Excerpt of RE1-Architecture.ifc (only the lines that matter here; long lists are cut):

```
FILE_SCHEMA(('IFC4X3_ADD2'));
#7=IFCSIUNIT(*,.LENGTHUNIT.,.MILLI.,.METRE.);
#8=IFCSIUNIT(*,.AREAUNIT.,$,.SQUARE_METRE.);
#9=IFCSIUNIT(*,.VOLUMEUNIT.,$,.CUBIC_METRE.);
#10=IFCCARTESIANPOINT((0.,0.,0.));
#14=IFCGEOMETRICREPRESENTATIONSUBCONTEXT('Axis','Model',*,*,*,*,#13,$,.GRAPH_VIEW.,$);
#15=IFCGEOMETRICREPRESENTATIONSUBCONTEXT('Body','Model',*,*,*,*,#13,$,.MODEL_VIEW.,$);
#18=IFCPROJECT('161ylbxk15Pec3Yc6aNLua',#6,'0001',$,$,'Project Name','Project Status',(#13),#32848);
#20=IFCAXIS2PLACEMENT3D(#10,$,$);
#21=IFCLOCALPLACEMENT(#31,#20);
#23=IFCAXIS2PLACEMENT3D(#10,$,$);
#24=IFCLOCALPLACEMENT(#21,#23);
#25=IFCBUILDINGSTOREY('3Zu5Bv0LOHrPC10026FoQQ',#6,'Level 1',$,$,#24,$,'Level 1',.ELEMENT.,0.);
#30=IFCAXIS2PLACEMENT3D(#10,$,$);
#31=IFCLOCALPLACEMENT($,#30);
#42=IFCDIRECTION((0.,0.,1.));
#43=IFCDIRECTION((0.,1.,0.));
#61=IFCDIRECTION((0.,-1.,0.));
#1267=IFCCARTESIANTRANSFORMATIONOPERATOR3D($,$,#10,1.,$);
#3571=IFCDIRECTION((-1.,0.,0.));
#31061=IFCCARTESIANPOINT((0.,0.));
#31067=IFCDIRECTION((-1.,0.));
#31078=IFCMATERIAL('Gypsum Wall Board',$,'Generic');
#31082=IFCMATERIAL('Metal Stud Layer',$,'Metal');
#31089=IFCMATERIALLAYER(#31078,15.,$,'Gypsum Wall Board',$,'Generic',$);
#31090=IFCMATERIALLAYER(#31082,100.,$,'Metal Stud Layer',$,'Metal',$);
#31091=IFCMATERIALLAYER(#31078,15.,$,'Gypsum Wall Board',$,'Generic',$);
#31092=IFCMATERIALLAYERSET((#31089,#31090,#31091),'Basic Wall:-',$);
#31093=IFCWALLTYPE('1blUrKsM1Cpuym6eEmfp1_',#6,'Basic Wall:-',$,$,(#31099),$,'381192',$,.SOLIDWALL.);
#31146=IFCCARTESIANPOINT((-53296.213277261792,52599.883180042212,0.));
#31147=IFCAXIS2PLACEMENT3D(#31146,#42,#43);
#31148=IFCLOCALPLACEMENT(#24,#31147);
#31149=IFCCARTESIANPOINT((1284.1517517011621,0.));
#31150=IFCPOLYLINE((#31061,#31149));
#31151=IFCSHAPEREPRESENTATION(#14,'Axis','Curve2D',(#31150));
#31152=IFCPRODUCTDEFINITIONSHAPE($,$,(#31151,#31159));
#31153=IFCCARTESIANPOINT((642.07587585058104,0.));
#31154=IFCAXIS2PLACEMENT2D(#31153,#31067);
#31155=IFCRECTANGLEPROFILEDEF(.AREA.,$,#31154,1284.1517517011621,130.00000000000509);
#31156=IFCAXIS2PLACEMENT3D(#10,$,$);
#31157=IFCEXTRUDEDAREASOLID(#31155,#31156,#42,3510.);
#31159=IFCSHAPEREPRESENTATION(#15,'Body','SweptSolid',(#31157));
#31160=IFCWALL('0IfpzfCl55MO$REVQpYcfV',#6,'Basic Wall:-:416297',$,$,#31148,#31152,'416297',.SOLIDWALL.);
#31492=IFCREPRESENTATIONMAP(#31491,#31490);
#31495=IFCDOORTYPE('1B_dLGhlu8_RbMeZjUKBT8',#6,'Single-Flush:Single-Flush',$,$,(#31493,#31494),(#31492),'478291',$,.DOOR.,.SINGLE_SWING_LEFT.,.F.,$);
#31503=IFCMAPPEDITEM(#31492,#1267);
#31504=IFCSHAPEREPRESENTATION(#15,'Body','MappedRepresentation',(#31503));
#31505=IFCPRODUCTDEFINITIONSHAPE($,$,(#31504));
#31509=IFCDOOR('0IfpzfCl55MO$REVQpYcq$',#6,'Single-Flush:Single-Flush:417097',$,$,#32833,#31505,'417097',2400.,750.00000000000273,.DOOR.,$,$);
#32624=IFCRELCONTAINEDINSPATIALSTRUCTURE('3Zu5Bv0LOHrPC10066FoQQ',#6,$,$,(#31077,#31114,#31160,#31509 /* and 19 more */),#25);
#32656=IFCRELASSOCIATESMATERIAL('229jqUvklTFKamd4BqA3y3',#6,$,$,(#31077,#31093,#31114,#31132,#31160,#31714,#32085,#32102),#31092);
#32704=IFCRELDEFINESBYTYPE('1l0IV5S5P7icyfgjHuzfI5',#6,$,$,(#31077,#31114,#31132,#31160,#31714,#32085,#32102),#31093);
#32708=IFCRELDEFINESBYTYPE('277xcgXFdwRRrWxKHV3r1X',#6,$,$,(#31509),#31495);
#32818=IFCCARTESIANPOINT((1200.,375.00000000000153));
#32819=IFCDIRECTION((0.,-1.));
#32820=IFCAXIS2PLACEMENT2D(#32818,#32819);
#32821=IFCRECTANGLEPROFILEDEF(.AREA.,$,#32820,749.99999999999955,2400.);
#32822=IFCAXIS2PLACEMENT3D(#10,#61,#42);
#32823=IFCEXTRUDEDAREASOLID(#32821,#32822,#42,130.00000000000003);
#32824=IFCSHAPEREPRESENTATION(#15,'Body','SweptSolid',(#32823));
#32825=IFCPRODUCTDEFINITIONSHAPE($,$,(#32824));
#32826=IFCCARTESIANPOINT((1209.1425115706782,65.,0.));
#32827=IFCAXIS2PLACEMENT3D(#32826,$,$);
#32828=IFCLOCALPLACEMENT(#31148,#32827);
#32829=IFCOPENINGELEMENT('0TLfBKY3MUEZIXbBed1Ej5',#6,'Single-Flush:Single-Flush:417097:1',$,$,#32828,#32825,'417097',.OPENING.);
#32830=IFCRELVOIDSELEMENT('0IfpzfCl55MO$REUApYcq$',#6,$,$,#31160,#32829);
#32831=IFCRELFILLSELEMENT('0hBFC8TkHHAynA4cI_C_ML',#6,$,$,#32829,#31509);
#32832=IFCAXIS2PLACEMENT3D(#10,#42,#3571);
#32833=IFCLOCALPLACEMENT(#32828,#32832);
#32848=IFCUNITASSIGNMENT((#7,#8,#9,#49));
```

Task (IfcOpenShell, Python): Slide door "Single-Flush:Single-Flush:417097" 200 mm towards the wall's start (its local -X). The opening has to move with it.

```python
import ifcopenshell
import ifcopenshell.api.geometry
import ifcopenshell.util.placement

model = ifcopenshell.open("RE1-Architecture.ifc")

door = model.by_guid("0IfpzfCl55MO$REVQpYcq$")
opening = door.FillsVoids[0].RelatingOpeningElement
wall = opening.VoidsElements[0].RelatingBuildingElement

wall_matrix = ifcopenshell.util.placement.get_local_placement(wall.ObjectPlacement)
shift = wall_matrix[:3, 0] * -200.0
before = ifcopenshell.util.placement.get_local_placement(door.ObjectPlacement)[:3, 3].copy()

# The door is placed relative to its opening, so it follows when the opening moves.
matrix = ifcopenshell.util.placement.get_local_placement(opening.ObjectPlacement)
matrix[:3, 3] += shift
ifcopenshell.api.geometry.edit_object_placement(
    model, product=opening, matrix=matrix, is_si=False, should_transform_children=True
)

after = ifcopenshell.util.placement.get_local_placement(door.ObjectPlacement)[:3, 3]
print("door moved by", (after - before).round(3) + 0.0)

model.write("RE1-Architecture_v2.ifc")
```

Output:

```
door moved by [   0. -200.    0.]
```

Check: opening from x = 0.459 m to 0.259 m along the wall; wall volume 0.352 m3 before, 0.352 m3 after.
